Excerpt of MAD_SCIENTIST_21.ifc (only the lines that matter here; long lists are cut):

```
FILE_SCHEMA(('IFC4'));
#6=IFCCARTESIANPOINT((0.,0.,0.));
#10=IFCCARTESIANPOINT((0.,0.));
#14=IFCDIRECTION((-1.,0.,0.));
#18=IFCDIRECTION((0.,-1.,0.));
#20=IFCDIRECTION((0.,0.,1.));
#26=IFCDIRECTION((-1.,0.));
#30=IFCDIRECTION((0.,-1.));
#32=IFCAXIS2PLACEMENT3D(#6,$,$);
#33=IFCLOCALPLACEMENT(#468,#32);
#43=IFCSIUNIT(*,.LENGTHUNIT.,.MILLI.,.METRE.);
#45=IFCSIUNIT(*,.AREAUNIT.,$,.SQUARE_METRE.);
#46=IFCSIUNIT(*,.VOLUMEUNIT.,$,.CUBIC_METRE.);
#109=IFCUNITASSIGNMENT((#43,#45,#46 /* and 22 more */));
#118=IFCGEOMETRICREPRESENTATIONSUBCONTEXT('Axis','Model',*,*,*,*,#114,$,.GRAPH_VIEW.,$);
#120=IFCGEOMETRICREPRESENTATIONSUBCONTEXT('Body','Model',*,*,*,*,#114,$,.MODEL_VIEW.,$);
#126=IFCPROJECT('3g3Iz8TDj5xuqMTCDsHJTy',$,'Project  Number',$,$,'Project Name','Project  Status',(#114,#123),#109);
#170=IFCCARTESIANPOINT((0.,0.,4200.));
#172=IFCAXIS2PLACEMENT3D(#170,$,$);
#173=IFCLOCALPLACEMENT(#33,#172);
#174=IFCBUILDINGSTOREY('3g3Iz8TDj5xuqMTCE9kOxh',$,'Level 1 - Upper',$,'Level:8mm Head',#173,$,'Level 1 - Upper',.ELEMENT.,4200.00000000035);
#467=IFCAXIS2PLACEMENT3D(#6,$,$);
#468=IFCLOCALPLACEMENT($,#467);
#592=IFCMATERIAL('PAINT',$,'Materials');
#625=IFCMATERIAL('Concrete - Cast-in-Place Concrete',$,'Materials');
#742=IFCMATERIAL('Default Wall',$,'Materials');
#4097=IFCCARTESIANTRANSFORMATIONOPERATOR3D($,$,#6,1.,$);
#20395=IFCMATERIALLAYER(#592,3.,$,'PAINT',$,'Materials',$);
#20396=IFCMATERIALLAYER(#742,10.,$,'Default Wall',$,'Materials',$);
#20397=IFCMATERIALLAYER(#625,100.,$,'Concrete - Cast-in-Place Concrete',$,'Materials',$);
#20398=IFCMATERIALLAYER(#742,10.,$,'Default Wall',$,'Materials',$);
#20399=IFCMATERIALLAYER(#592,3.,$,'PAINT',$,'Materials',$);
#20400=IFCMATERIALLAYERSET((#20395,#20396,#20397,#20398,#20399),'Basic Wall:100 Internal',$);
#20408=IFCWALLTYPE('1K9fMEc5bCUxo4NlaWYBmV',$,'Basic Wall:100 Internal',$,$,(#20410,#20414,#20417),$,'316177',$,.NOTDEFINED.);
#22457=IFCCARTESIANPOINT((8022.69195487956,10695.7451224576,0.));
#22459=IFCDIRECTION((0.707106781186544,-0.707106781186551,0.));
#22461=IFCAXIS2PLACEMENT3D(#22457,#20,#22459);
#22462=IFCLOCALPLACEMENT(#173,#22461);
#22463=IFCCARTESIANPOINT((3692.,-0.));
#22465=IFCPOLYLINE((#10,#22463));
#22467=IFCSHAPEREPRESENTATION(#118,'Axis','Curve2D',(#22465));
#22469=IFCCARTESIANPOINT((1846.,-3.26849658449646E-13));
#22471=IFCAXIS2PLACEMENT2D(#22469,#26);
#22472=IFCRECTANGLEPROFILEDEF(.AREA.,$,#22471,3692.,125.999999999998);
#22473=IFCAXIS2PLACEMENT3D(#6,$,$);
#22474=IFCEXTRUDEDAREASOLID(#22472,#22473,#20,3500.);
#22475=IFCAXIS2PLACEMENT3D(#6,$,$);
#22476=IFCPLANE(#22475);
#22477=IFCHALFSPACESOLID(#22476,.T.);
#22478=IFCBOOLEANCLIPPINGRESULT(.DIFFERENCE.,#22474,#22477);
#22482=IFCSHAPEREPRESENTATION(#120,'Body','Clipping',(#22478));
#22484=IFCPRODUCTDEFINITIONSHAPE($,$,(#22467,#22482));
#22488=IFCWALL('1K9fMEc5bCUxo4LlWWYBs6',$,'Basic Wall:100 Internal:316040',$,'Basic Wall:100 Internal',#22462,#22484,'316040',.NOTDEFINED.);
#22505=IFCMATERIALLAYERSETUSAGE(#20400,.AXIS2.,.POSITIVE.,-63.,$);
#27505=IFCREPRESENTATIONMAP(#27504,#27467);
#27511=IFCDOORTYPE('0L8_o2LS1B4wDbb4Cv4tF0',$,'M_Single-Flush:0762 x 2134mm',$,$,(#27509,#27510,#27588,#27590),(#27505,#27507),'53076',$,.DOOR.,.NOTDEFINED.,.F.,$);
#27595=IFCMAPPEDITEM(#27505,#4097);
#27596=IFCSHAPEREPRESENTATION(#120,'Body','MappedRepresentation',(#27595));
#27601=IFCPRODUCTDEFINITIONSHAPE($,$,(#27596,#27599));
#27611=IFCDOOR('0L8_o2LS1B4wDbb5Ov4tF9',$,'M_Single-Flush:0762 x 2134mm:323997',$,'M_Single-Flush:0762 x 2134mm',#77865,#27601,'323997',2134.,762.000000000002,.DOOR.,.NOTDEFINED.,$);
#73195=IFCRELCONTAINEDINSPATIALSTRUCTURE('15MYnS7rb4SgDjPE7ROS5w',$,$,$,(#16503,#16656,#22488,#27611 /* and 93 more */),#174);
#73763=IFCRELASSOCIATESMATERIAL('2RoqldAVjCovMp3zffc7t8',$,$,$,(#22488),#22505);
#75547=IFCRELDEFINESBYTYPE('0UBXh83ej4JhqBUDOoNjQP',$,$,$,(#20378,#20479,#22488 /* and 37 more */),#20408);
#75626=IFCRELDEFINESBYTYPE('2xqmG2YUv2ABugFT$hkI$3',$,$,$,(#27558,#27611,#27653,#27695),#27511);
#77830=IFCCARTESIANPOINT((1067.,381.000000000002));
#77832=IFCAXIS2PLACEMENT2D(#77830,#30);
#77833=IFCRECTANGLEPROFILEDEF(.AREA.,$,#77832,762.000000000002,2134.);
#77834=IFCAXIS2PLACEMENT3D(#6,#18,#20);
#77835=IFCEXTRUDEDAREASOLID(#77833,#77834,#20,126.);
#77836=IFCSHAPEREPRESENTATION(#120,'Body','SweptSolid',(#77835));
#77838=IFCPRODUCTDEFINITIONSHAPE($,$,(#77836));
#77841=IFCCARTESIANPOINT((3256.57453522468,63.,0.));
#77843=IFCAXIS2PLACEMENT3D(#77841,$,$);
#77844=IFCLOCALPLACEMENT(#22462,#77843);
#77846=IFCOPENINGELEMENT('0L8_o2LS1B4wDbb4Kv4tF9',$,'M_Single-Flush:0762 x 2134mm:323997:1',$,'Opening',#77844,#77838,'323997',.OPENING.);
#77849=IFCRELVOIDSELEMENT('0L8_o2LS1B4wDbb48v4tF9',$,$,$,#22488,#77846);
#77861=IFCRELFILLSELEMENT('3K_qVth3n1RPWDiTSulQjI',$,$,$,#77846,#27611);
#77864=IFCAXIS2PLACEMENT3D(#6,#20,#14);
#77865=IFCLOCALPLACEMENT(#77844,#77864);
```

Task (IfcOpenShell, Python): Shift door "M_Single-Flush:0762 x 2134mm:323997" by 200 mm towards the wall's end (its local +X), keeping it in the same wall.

```python
import ifcopenshell
import ifcopenshell.api.geometry
import ifcopenshell.util.placement

model = ifcopenshell.open("MAD_SCIENTIST_21.ifc")

door = model.by_guid("0L8_o2LS1B4wDbb5Ov4tF9")
opening = door.FillsVoids[0].RelatingOpeningElement
wall = opening.VoidsElements[0].RelatingBuildingElement

wall_matrix = ifcopenshell.util.placement.get_local_placement(wall.ObjectPlacement)
shift = wall_matrix[:3, 0] * 200.0
before = ifcopenshell.util.placement.get_local_placement(door.ObjectPlacement)[:3, 3].copy()

# The door is placed relative to its opening, so it follows when the opening moves.
matrix = ifcopenshell.util.placement.get_local_placement(opening.ObjectPlacement)
matrix[:3, 3] += shift
ifcopenshell.api.geometry.edit_object_placement(
    model, product=opening, matrix=matrix, is_si=False, should_transform_children=True
)

after = ifcopenshell.util.placement.get_local_placement(door.ObjectPlacement)[:3, 3]
print("door moved by", (after - before).round(3) + 0.0)

model.write("MAD_SCIENTIST_21_v2.ifc")
```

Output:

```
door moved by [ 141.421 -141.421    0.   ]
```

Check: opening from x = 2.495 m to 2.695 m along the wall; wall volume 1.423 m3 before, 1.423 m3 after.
